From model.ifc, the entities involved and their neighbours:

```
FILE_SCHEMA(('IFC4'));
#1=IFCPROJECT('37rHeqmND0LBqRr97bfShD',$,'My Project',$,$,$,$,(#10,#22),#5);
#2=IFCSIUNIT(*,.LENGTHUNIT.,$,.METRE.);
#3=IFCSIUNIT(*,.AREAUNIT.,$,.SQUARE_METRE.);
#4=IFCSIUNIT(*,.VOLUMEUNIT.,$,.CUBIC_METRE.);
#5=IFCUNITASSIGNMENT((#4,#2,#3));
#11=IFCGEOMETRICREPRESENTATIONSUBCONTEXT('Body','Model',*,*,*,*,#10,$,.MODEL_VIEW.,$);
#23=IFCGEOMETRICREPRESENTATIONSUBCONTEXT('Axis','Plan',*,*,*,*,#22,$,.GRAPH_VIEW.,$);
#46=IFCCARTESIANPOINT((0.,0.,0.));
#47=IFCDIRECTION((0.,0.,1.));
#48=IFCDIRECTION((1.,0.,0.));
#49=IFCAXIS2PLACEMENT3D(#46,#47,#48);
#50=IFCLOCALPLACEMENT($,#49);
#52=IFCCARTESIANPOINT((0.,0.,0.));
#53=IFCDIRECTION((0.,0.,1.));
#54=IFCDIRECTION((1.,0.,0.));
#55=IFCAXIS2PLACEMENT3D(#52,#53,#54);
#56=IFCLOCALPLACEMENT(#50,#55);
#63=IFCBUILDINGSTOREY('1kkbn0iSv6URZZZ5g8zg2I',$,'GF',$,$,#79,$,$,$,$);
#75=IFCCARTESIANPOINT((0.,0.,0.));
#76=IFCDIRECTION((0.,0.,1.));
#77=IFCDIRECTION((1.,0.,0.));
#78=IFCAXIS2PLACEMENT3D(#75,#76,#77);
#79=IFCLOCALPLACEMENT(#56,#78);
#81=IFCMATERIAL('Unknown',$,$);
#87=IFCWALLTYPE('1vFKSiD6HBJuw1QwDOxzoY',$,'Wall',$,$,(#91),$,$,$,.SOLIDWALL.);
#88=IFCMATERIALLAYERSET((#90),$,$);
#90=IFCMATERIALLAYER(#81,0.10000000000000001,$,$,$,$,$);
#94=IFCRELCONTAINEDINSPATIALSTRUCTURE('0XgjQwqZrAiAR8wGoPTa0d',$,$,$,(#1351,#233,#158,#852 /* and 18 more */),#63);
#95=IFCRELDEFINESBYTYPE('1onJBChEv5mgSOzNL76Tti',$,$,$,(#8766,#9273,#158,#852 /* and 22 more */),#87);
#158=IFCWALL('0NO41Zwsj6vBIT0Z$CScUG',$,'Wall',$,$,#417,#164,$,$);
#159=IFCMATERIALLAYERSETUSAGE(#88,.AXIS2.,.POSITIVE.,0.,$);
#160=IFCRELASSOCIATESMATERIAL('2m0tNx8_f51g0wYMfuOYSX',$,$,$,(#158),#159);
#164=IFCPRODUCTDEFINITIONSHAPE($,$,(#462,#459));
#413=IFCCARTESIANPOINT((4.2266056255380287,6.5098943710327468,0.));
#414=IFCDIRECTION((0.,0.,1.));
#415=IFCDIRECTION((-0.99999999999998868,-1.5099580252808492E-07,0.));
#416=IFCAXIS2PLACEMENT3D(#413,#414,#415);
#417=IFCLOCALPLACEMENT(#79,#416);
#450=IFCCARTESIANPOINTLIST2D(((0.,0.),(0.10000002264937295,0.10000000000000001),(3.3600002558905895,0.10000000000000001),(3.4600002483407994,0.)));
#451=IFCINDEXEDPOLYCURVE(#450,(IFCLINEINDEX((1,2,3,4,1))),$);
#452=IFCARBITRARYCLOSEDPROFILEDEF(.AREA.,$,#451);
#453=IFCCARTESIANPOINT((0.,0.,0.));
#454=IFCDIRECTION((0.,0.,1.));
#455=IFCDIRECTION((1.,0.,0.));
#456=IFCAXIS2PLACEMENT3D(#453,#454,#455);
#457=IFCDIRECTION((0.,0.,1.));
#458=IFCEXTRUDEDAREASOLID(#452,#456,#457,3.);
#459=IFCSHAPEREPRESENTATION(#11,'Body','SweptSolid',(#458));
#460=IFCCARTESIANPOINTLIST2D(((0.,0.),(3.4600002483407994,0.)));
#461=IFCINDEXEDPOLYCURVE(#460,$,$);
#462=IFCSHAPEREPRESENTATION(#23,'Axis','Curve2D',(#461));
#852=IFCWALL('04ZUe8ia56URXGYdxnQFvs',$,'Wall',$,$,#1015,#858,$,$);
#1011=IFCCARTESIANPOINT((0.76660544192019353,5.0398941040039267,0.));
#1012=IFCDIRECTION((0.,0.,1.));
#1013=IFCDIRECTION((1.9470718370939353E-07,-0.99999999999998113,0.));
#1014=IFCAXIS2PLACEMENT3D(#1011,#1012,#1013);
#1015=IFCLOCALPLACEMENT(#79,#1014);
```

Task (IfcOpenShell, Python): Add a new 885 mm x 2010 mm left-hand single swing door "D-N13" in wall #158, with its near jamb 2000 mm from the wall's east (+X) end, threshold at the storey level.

```python
import numpy as np
import ifcopenshell
import ifcopenshell.api.feature
import ifcopenshell.api.geometry
import ifcopenshell.api.root
import ifcopenshell.api.spatial
import ifcopenshell.geom
import ifcopenshell.util.element
import ifcopenshell.util.placement
import ifcopenshell.util.representation
import ifcopenshell.util.shape
import ifcopenshell.util.unit

model = ifcopenshell.open("model.ifc")
unit_scale = ifcopenshell.util.unit.calculate_unit_scale(model)
settings = ifcopenshell.geom.settings()


def volume(element):
    """Net volume in cubic metres, openings subtracted."""
    shape = ifcopenshell.geom.create_shape(settings, element)
    return ifcopenshell.util.shape.get_volume(shape.geometry)


wall = model.by_guid("0NO41Zwsj6vBIT0Z$CScUG")
storey = ifcopenshell.util.element.get_container(wall, ifc_class="IfcBuildingStorey")
context = ifcopenshell.util.representation.get_context(model, "Model", "Body", "MODEL_VIEW")
before = volume(wall)

width, height, from_end, sill = 0.885, 2.01, 2, 0.0  # metres

# The wall runs along its own X axis, and the end named is its -X end.
wall_shape = ifcopenshell.geom.create_shape(settings, wall)
x, y, z = ifcopenshell.util.shape.get_vertices(wall_shape.geometry).T
start = x.min() + from_end
face, thickness = float(y.min()), float(y.max() - y.min())
wall_matrix = ifcopenshell.util.placement.get_local_placement(wall.ObjectPlacement)
level = ifcopenshell.util.placement.get_local_placement(storey.ObjectPlacement)[2, 3]


def in_wall(x, y):
    """Placement at x, y metres in the wall's axes, at sill height."""
    matrix = wall_matrix.copy()
    matrix[:, 3] = wall_matrix @ np.array([x / unit_scale, y / unit_scale, 0.0, 1.0])
    matrix[2, 3] = level + sill / unit_scale
    return matrix


# Opening: a box that overshoots both wall faces by 50 mm.
opening = ifcopenshell.api.root.create_entity(model, ifc_class="IfcOpeningElement", predefined_type="OPENING")
box = ifcopenshell.api.geometry.add_wall_representation(
    model, context=context, length=width, height=height, thickness=thickness + 0.1
)
ifcopenshell.api.geometry.assign_representation(model, product=opening, representation=box)
ifcopenshell.api.geometry.edit_object_placement(model, product=opening, matrix=in_wall(start, face - 0.05), is_si=False)
ifcopenshell.api.feature.add_feature(model, feature=opening, element=wall)

door = ifcopenshell.api.root.create_entity(model, ifc_class="IfcDoor", name="D-N13", predefined_type="DOOR")
door.OverallWidth, door.OverallHeight = width / unit_scale, height / unit_scale
door.OperationType = "SINGLE_SWING_LEFT"
body = ifcopenshell.api.geometry.add_door_representation(
    model,
    context=context,
    overall_width=door.OverallWidth,
    overall_height=door.OverallHeight,
    operation_type="SINGLE_SWING_LEFT",
    lining_properties={"LiningDepth": thickness / unit_scale, "ThresholdDepth": thickness / unit_scale},
)
ifcopenshell.api.geometry.assign_representation(model, product=door, representation=body)
ifcopenshell.api.spatial.assign_container(model, products=[door], relating_structure=storey)
ifcopenshell.api.feature.add_filling(model, opening=opening, element=door)

# The lining spans the wall, so the door starts at the wall face.
ifcopenshell.api.geometry.edit_object_placement(model, product=door, matrix=in_wall(start, face), is_si=False)

after = volume(wall)

print(f"wall volume {before:.3f} -> {after:.3f} m3")

model.write("model_v2.ifc")
```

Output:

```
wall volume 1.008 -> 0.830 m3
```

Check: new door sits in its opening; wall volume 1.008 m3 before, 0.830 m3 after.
